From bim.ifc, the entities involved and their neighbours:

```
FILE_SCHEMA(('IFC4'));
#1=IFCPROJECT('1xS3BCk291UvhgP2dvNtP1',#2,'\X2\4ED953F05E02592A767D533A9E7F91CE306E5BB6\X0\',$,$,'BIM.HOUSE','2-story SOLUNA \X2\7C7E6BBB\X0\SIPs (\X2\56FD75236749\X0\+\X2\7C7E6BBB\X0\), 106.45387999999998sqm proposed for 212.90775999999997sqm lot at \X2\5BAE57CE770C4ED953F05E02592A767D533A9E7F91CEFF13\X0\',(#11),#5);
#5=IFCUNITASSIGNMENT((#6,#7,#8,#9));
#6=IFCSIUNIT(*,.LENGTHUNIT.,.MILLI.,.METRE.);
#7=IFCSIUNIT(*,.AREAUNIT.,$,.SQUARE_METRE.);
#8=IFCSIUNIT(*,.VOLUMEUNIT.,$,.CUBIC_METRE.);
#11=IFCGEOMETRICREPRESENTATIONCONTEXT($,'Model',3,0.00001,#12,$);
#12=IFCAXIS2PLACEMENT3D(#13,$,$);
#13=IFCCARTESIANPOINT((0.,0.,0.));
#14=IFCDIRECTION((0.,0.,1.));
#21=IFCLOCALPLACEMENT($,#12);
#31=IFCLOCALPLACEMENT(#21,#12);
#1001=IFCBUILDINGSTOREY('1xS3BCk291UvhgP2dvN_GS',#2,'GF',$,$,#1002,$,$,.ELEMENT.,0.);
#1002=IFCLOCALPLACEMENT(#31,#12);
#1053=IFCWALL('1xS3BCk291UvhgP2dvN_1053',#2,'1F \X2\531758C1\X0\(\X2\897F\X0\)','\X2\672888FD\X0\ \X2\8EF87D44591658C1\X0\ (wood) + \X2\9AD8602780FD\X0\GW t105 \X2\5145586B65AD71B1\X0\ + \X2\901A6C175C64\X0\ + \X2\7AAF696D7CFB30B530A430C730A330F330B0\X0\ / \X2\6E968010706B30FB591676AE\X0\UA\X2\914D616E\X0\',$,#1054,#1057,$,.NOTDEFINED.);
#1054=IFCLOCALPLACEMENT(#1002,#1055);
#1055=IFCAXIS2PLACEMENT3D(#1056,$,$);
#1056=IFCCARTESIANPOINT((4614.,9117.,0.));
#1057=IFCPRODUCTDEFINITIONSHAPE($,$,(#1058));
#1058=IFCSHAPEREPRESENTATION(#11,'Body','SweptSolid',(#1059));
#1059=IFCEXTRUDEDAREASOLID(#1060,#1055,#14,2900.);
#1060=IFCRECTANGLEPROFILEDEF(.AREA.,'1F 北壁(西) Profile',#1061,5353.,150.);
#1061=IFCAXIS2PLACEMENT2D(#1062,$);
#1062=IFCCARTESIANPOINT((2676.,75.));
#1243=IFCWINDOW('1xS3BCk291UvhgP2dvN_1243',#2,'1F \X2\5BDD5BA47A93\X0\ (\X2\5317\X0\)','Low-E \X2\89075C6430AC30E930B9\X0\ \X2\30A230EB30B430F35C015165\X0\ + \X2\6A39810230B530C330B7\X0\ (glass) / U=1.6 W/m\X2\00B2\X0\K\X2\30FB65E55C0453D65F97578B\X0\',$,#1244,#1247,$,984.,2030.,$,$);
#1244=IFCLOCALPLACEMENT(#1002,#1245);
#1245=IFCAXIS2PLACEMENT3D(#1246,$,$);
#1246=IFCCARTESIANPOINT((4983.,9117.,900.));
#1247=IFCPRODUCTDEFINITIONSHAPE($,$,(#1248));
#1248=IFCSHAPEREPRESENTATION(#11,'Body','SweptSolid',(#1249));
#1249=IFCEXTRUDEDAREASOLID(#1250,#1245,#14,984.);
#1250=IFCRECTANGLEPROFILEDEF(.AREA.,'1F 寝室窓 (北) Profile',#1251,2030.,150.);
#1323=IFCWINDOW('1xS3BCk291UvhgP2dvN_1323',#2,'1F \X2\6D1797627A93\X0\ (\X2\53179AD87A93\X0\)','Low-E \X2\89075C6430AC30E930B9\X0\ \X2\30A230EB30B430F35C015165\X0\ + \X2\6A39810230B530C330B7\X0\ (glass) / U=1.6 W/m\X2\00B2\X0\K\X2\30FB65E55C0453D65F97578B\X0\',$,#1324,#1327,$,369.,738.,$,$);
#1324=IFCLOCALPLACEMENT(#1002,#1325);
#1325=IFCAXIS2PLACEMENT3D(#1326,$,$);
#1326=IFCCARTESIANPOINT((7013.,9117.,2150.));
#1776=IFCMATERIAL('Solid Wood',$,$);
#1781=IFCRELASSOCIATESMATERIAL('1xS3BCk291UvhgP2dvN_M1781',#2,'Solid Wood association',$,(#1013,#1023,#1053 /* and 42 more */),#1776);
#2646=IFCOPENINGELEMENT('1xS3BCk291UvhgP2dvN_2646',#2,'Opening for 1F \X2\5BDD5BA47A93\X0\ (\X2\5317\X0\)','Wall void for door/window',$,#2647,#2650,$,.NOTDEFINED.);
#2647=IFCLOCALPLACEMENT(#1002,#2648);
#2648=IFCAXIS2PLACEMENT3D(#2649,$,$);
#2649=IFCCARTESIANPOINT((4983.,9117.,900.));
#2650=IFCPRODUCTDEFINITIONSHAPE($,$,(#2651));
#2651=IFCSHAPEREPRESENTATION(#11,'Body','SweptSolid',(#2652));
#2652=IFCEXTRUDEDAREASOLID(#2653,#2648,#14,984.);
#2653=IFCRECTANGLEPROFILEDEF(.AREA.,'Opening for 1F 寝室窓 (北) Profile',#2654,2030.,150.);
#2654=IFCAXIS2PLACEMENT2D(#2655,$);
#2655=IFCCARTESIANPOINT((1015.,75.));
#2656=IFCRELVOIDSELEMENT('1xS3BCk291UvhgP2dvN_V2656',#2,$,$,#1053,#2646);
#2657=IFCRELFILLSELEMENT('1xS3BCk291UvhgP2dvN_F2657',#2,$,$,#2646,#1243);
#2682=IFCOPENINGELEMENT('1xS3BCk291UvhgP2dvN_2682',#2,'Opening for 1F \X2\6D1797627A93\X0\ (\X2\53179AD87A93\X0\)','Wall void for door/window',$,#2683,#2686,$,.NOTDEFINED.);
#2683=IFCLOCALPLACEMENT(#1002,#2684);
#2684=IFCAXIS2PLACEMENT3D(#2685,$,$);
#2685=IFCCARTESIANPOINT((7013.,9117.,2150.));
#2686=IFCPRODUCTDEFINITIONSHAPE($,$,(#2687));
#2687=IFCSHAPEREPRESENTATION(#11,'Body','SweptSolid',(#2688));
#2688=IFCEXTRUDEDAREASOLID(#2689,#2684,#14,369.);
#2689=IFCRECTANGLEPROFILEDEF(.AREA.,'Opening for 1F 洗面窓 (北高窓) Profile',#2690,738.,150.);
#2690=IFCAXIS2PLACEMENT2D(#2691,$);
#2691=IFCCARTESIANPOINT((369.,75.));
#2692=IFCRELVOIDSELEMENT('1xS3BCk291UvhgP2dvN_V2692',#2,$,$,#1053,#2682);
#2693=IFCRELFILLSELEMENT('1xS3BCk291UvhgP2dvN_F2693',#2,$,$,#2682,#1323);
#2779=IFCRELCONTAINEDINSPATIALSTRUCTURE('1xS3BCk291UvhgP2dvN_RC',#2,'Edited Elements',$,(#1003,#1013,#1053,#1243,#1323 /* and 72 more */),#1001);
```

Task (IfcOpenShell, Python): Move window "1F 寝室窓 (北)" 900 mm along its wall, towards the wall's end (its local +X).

```python
import ifcopenshell
import ifcopenshell.api.geometry
import ifcopenshell.util.placement
import ifcopenshell.util.unit

model = ifcopenshell.open("bim.ifc")
unit_scale = ifcopenshell.util.unit.calculate_unit_scale(model)

window = model.by_guid("1xS3BCk291UvhgP2dvN_1243")
opening = window.FillsVoids[0].RelatingOpeningElement
wall = opening.VoidsElements[0].RelatingBuildingElement

wall_matrix = ifcopenshell.util.placement.get_local_placement(wall.ObjectPlacement)
shift = wall_matrix[:3, 0] * 0.9 / unit_scale
before = ifcopenshell.util.placement.get_local_placement(window.ObjectPlacement)[:3, 3].copy()

# The window is not placed relative to its opening, so move both.
for product in (opening, window):
    matrix = ifcopenshell.util.placement.get_local_placement(product.ObjectPlacement)
    matrix[:3, 3] += shift
    ifcopenshell.api.geometry.edit_object_placement(model, product=product, matrix=matrix, is_si=False)

after = ifcopenshell.util.placement.get_local_placement(window.ObjectPlacement)[:3, 3]
print("window moved by", (after - before).round(3) + 0.0)

model.write("bim_updated.ifc")
```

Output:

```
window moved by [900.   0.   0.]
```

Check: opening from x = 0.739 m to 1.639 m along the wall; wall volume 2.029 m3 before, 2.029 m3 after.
